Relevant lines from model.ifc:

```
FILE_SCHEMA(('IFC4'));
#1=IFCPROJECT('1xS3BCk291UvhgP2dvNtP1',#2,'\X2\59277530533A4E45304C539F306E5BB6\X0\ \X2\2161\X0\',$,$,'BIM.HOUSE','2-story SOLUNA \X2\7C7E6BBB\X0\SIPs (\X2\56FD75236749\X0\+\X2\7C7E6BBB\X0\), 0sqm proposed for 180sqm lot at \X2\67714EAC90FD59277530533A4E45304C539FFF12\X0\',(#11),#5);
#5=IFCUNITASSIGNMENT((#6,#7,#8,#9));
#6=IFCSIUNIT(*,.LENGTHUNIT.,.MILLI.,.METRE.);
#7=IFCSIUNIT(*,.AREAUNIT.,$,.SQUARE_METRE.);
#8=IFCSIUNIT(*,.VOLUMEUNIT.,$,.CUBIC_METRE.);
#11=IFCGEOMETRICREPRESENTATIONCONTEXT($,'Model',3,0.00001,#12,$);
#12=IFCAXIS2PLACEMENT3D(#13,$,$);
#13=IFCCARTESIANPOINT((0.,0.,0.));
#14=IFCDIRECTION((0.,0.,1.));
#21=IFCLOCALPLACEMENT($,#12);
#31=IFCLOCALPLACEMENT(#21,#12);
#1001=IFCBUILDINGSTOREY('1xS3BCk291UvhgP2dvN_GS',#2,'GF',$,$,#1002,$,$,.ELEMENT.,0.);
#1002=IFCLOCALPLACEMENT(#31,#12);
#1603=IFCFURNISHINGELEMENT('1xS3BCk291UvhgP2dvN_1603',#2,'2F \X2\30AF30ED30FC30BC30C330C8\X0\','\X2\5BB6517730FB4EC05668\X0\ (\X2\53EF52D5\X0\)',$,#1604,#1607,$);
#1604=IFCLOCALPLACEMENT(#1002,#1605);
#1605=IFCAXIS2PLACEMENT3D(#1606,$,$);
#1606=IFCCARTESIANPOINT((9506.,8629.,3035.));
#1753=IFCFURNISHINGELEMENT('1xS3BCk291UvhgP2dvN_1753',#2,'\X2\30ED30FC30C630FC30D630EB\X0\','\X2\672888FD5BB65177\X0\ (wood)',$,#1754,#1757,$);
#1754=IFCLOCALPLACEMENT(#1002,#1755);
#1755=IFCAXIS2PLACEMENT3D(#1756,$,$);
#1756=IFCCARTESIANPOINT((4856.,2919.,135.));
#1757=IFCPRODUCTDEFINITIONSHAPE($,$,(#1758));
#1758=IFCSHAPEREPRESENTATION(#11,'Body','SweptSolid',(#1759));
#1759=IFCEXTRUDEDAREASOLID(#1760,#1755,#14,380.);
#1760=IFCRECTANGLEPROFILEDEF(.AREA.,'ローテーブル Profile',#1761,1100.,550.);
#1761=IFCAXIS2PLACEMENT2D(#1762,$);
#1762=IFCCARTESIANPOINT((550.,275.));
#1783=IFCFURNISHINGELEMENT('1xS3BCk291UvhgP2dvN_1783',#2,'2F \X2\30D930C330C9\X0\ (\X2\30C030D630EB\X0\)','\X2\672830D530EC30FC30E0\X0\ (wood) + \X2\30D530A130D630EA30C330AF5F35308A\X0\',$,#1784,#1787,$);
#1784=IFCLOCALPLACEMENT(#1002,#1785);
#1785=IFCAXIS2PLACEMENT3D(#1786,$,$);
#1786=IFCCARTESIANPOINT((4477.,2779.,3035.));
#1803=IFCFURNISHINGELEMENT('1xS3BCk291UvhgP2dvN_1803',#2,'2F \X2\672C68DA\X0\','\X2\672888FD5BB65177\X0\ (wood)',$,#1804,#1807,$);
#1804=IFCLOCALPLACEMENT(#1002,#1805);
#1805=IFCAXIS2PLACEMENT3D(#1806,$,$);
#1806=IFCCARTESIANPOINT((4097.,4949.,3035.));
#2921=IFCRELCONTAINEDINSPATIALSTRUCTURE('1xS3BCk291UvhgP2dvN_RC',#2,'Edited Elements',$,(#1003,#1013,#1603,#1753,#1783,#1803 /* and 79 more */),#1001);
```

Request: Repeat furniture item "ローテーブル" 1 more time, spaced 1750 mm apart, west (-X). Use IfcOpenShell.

```python
import numpy as np
import ifcopenshell
import ifcopenshell.api.geometry
import ifcopenshell.api.root
import ifcopenshell.util.element
import ifcopenshell.util.placement

model = ifcopenshell.open("model.ifc")


def reuse_history(source, copy):
    """copy_class also copies each property set's owner history, people and application; keep the originals."""
    for rel in copy.IsDefinedBy:
        if rel.is_a("IfcRelDefinesByProperties") and (history := rel.RelatingPropertyDefinition.OwnerHistory):
            rel.RelatingPropertyDefinition.OwnerHistory = source.OwnerHistory
            ifcopenshell.util.element.remove_deep2(model, history)


source = model.by_id(1753)
base = ifcopenshell.util.placement.get_local_placement(source.ObjectPlacement)
step = np.array([-1.0, 0.0, 0.0]) * 1750.0

for i in range(1, 2):
    copy = ifcopenshell.api.root.copy_class(model, product=source)
    copy.Representation = ifcopenshell.util.element.copy_deep(
        model, source.Representation, exclude=["IfcGeometricRepresentationContext", "IfcRepresentationMap"]
    )
    reuse_history(source, copy)
    matrix = base.copy()
    matrix[:3, 3] += i * step
    print("added at", matrix[:3, 3].round(3) + 0.0)
    ifcopenshell.api.geometry.edit_object_placement(model, product=copy, matrix=matrix, is_si=False)

model.write("model_v2.ifc")
```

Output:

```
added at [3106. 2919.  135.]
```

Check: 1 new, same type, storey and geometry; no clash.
